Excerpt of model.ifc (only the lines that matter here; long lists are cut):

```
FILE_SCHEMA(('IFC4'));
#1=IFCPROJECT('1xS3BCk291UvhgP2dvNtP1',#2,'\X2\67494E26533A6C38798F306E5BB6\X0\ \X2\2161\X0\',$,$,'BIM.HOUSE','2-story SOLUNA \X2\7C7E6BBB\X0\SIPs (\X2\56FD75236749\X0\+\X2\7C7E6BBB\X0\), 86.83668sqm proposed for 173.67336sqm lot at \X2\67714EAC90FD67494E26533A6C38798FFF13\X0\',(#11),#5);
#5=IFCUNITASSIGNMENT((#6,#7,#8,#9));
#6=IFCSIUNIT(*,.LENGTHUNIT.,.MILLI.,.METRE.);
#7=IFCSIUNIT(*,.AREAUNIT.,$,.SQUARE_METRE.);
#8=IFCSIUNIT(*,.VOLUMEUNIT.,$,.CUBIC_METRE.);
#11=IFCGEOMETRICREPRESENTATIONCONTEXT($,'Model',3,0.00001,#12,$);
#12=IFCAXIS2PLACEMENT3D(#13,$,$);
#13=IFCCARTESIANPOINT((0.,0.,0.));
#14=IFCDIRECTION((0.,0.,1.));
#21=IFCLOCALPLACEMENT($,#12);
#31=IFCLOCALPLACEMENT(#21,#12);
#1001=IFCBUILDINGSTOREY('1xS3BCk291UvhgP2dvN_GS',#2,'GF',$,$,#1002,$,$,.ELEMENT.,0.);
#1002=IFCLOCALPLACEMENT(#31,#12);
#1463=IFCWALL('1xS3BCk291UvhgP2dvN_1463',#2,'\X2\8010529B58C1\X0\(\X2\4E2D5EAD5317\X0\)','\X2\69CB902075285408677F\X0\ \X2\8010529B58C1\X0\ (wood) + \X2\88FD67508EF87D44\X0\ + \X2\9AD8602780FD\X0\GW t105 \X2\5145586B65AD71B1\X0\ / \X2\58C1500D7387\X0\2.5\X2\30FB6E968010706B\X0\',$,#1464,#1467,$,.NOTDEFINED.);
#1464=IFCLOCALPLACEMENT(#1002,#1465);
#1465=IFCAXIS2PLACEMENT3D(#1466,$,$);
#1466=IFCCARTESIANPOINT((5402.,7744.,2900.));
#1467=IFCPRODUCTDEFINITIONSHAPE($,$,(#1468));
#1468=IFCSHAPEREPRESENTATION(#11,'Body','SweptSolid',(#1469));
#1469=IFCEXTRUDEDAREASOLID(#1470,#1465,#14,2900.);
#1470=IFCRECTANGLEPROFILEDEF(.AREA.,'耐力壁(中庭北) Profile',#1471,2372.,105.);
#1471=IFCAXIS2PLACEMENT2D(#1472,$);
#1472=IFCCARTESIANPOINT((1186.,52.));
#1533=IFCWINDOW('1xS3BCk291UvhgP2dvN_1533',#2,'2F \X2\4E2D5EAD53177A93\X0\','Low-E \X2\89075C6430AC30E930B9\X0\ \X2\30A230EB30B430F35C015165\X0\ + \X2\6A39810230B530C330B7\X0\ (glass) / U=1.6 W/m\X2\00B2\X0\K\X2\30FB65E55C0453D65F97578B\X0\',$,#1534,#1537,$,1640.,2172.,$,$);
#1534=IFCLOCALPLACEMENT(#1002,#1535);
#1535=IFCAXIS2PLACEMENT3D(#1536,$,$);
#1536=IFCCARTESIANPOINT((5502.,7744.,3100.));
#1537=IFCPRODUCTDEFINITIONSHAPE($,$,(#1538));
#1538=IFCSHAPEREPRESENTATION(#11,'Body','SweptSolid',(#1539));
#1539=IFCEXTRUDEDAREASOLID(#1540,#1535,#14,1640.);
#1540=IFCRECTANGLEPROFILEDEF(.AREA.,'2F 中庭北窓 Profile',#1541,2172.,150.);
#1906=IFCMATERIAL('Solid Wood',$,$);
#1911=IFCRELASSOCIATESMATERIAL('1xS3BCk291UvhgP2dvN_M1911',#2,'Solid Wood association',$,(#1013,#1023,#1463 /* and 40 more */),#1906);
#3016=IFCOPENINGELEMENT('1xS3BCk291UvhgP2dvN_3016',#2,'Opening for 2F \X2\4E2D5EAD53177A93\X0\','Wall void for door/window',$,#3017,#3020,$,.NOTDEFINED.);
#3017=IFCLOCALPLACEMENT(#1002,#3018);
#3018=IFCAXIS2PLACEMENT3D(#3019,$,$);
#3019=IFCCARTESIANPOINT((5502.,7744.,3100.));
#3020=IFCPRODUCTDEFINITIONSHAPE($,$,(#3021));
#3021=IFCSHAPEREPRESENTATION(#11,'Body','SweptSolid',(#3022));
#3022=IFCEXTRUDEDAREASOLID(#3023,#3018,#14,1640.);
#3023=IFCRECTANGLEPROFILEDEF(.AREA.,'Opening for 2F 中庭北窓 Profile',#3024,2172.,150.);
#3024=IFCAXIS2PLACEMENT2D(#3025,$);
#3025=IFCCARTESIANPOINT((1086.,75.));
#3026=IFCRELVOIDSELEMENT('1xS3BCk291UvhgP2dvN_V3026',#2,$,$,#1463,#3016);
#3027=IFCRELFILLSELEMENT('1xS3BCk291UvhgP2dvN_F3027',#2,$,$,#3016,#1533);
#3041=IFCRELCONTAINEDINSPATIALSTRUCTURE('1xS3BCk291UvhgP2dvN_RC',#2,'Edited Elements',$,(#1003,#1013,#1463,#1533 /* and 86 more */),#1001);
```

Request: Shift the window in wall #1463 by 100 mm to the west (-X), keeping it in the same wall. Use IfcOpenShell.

```python
import ifcopenshell
import ifcopenshell.api.geometry
import ifcopenshell.util.placement
import ifcopenshell.util.unit

model = ifcopenshell.open("model.ifc")
unit_scale = ifcopenshell.util.unit.calculate_unit_scale(model)

window = model.by_id(1533)
opening = window.FillsVoids[0].RelatingOpeningElement
wall = opening.VoidsElements[0].RelatingBuildingElement

wall_matrix = ifcopenshell.util.placement.get_local_placement(wall.ObjectPlacement)
shift = wall_matrix[:3, 0] * -0.1 / unit_scale
before = ifcopenshell.util.placement.get_local_placement(window.ObjectPlacement)[:3, 3].copy()

# The window is not placed relative to its opening, so move both.
for product in (opening, window):
    matrix = ifcopenshell.util.placement.get_local_placement(product.ObjectPlacement)
    matrix[:3, 3] += shift
    ifcopenshell.api.geometry.edit_object_placement(model, product=product, matrix=matrix, is_si=False)

after = ifcopenshell.util.placement.get_local_placement(window.ObjectPlacement)[:3, 3]
print("window moved by", (after - before).round(3) + 0.0)

model.write("model-out.ifc")
```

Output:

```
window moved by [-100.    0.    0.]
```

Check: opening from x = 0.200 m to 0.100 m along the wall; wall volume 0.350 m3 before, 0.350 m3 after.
